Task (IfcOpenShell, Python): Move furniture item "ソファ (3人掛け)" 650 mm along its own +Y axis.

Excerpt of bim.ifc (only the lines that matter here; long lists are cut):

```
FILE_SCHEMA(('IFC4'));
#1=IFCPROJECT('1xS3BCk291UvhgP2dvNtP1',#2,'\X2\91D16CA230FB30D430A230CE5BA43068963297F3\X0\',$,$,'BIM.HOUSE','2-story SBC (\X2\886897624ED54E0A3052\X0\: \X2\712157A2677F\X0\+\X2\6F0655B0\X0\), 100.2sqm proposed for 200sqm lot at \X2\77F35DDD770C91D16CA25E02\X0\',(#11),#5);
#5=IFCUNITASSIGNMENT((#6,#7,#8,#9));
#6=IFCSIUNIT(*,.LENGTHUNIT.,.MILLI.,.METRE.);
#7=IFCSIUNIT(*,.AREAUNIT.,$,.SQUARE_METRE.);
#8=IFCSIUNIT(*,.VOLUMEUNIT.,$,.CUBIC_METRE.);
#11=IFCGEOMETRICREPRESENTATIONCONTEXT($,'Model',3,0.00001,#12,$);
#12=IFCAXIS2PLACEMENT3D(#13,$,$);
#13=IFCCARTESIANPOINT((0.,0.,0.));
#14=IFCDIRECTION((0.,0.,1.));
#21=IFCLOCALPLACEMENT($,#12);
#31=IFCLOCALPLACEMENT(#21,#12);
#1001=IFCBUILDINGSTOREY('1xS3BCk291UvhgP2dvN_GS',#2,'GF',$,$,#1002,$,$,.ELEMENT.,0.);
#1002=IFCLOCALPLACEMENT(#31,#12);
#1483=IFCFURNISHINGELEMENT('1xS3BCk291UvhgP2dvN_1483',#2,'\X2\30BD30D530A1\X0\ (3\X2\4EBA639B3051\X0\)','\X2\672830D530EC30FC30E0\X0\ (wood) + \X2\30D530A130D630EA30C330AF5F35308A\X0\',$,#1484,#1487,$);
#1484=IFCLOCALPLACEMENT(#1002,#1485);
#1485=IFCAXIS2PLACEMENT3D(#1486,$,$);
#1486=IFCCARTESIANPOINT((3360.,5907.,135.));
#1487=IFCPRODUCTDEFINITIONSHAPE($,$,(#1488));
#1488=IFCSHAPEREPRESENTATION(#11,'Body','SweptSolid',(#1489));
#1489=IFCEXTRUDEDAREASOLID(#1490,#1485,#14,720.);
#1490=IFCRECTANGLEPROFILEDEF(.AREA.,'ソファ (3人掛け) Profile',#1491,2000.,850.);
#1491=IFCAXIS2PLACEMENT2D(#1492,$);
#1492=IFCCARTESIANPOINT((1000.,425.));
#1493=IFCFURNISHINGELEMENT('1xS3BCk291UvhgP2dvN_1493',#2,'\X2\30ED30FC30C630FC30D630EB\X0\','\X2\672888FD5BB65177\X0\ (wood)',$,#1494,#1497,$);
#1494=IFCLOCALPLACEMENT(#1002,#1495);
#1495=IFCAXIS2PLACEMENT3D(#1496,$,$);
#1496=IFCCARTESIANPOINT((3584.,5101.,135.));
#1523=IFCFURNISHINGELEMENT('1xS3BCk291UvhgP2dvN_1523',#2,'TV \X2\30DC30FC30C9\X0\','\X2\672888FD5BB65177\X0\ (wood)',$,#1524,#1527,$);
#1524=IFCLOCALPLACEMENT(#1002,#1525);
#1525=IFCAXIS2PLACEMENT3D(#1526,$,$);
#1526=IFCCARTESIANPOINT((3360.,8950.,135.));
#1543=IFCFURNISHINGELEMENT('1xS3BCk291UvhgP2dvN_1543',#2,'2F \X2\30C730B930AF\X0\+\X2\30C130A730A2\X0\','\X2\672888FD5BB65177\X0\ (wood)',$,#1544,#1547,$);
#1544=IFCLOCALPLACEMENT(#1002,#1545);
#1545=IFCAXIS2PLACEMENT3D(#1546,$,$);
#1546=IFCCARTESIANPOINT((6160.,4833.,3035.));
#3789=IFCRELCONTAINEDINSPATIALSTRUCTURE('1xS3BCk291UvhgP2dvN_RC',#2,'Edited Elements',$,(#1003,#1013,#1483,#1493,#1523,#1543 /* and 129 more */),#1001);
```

```python
import ifcopenshell
import ifcopenshell.api.geometry
import ifcopenshell.util.placement

model = ifcopenshell.open("bim.ifc")

item = model.by_guid("1xS3BCk291UvhgP2dvN_1483")
matrix = ifcopenshell.util.placement.get_local_placement(item.ObjectPlacement)
matrix[:3, 3] += matrix[:3, 1] * 650.0
ifcopenshell.api.geometry.edit_object_placement(model, product=item, matrix=matrix, is_si=False)

print(ifcopenshell.util.placement.get_local_placement(item.ObjectPlacement).round(3) + 0.0)

model.write("bim_rev.ifc")
```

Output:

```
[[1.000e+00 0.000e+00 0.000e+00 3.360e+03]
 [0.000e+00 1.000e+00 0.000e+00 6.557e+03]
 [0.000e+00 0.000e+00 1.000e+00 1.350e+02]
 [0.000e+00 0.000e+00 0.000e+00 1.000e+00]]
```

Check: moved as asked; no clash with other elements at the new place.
